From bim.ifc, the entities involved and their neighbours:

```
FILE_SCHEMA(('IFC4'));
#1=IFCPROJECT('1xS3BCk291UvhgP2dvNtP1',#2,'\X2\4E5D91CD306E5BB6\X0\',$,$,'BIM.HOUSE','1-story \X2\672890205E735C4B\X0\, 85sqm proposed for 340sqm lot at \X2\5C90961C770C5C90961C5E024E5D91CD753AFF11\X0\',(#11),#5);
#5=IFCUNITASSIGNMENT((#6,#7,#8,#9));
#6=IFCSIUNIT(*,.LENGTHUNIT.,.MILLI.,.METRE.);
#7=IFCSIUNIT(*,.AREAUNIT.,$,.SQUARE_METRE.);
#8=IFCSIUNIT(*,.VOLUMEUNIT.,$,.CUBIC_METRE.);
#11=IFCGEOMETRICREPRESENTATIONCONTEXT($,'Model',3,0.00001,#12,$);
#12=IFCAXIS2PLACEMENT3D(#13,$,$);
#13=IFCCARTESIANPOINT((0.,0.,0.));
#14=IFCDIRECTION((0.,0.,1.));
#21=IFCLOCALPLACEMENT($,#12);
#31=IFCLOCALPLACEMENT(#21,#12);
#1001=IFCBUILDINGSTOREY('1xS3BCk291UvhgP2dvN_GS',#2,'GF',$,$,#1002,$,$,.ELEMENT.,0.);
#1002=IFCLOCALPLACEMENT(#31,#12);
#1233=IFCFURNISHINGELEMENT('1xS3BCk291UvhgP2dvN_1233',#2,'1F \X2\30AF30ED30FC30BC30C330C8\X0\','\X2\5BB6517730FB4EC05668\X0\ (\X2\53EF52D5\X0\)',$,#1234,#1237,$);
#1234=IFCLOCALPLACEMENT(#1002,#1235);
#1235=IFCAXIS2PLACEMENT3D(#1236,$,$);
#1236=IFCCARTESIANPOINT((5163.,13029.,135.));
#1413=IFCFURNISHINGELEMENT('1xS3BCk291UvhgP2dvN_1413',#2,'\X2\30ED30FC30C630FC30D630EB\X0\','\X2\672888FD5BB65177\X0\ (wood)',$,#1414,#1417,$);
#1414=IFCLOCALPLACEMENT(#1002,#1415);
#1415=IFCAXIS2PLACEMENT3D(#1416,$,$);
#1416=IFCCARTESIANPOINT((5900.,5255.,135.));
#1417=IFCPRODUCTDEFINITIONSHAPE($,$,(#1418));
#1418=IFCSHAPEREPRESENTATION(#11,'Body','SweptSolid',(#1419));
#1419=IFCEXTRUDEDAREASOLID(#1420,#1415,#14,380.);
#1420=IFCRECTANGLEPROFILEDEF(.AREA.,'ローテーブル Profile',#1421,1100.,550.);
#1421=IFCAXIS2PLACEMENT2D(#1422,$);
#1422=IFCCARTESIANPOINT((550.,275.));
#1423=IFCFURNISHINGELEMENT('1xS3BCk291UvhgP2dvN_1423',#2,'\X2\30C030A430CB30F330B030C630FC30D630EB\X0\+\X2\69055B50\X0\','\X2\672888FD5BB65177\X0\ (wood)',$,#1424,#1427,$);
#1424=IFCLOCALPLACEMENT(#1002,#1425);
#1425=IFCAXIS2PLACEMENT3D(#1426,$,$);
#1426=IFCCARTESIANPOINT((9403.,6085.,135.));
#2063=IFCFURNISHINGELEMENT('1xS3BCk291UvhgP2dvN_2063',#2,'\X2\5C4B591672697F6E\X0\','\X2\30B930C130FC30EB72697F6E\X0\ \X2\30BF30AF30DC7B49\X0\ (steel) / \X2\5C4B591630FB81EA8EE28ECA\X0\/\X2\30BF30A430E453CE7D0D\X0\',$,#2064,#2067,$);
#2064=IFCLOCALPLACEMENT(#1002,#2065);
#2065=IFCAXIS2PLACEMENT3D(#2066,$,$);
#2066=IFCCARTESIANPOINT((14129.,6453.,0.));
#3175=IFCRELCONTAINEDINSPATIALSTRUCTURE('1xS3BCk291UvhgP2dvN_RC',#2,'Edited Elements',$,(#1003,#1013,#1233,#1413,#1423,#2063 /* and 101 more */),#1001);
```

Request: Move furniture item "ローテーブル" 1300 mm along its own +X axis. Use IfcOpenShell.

```python
import ifcopenshell
import ifcopenshell.api.geometry
import ifcopenshell.util.placement
import ifcopenshell.util.unit

model = ifcopenshell.open("bim.ifc")
unit_scale = ifcopenshell.util.unit.calculate_unit_scale(model)

item = model.by_id(1413)
matrix = ifcopenshell.util.placement.get_local_placement(item.ObjectPlacement)
matrix[:3, 3] += matrix[:3, 0] * 1.3 / unit_scale
ifcopenshell.api.geometry.edit_object_placement(model, product=item, matrix=matrix, is_si=False)

print(ifcopenshell.util.placement.get_local_placement(item.ObjectPlacement).round(3) + 0.0)

model.write("bim_edited.ifc")
```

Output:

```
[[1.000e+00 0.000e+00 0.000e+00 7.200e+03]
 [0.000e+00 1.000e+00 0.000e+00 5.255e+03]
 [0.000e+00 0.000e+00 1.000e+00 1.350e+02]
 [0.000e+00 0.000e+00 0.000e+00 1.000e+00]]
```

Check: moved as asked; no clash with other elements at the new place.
